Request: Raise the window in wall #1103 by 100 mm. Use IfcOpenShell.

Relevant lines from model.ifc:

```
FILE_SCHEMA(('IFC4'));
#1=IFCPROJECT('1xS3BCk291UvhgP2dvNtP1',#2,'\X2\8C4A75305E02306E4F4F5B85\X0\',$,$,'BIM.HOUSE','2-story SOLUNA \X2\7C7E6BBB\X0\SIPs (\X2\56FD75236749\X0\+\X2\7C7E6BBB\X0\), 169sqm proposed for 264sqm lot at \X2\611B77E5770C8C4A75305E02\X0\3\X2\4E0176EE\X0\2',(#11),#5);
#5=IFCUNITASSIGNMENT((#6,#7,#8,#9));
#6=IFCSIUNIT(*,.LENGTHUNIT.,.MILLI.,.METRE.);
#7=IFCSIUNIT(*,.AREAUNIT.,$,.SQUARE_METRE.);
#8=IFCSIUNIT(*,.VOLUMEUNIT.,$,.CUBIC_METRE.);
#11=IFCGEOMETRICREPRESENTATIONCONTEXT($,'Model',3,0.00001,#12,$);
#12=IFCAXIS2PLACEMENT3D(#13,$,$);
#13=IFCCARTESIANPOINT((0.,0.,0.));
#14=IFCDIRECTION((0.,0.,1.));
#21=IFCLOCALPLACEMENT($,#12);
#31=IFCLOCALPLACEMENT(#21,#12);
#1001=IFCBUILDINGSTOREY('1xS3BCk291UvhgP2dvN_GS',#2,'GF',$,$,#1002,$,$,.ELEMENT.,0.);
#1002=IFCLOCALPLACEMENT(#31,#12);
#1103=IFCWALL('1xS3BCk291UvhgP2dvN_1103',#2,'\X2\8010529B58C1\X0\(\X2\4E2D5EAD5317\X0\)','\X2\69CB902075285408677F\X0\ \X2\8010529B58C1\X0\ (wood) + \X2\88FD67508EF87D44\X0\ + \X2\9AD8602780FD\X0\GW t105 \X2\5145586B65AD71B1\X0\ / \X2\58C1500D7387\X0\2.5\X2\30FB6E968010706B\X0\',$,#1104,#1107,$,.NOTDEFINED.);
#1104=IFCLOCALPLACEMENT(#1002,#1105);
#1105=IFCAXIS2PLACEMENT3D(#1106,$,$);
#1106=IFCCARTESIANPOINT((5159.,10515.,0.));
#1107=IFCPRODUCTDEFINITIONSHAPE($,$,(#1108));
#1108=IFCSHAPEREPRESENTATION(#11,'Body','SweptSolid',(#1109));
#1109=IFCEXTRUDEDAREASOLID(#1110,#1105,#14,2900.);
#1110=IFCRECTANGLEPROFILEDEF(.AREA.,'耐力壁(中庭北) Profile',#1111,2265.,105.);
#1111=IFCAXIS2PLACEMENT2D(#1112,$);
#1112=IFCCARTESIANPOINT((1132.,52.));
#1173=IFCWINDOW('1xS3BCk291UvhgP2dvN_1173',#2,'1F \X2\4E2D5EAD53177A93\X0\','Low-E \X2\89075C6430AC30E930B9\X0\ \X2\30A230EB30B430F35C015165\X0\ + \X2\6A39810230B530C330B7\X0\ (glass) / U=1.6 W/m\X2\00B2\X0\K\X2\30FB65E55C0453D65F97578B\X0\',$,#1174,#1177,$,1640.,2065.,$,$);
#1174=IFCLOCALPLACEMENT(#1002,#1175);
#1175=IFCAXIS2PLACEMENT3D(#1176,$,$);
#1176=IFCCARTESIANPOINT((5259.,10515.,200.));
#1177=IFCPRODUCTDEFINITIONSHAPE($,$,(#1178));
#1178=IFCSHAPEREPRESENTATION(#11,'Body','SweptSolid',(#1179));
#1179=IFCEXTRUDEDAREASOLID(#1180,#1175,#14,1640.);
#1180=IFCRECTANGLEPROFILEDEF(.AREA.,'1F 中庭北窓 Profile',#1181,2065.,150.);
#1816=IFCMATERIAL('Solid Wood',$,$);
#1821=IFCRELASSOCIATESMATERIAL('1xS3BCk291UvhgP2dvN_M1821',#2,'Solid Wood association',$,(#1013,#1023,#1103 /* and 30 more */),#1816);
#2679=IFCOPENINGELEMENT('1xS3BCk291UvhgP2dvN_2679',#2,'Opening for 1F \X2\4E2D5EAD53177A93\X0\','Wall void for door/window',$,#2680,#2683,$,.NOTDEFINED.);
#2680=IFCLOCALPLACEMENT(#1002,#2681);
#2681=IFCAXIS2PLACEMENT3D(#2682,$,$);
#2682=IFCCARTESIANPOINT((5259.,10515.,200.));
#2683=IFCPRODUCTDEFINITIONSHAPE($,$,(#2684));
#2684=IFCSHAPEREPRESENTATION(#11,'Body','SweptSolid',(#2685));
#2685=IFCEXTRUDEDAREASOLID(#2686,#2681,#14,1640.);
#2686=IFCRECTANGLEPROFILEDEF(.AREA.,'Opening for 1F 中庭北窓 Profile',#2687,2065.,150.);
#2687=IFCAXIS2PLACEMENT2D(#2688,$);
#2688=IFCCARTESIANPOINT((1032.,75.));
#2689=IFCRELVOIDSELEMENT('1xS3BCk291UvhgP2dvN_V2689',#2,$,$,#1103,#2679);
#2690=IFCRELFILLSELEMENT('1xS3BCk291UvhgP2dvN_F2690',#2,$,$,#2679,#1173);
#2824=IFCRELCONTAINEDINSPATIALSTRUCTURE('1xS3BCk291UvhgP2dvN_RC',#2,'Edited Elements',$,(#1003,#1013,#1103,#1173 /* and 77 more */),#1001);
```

```python
import numpy as np
import ifcopenshell
import ifcopenshell.api.geometry
import ifcopenshell.util.placement
import ifcopenshell.util.unit

model = ifcopenshell.open("model.ifc")
unit_scale = ifcopenshell.util.unit.calculate_unit_scale(model)

window = model.by_id(1173)
opening = window.FillsVoids[0].RelatingOpeningElement
dz = 0.1 / unit_scale

shift = np.array([0.0, 0.0, dz])
# The window is not placed relative to its opening, so move both.
for product in (opening, window):
    matrix = ifcopenshell.util.placement.get_local_placement(product.ObjectPlacement)
    matrix[:3, 3] += shift
    ifcopenshell.api.geometry.edit_object_placement(model, product=product, matrix=matrix, is_si=False)

print(f"moved by {dz * unit_scale:+.3f} m")

model.write("model_v2.ifc")
```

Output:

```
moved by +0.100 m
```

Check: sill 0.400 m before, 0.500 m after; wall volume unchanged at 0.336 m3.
